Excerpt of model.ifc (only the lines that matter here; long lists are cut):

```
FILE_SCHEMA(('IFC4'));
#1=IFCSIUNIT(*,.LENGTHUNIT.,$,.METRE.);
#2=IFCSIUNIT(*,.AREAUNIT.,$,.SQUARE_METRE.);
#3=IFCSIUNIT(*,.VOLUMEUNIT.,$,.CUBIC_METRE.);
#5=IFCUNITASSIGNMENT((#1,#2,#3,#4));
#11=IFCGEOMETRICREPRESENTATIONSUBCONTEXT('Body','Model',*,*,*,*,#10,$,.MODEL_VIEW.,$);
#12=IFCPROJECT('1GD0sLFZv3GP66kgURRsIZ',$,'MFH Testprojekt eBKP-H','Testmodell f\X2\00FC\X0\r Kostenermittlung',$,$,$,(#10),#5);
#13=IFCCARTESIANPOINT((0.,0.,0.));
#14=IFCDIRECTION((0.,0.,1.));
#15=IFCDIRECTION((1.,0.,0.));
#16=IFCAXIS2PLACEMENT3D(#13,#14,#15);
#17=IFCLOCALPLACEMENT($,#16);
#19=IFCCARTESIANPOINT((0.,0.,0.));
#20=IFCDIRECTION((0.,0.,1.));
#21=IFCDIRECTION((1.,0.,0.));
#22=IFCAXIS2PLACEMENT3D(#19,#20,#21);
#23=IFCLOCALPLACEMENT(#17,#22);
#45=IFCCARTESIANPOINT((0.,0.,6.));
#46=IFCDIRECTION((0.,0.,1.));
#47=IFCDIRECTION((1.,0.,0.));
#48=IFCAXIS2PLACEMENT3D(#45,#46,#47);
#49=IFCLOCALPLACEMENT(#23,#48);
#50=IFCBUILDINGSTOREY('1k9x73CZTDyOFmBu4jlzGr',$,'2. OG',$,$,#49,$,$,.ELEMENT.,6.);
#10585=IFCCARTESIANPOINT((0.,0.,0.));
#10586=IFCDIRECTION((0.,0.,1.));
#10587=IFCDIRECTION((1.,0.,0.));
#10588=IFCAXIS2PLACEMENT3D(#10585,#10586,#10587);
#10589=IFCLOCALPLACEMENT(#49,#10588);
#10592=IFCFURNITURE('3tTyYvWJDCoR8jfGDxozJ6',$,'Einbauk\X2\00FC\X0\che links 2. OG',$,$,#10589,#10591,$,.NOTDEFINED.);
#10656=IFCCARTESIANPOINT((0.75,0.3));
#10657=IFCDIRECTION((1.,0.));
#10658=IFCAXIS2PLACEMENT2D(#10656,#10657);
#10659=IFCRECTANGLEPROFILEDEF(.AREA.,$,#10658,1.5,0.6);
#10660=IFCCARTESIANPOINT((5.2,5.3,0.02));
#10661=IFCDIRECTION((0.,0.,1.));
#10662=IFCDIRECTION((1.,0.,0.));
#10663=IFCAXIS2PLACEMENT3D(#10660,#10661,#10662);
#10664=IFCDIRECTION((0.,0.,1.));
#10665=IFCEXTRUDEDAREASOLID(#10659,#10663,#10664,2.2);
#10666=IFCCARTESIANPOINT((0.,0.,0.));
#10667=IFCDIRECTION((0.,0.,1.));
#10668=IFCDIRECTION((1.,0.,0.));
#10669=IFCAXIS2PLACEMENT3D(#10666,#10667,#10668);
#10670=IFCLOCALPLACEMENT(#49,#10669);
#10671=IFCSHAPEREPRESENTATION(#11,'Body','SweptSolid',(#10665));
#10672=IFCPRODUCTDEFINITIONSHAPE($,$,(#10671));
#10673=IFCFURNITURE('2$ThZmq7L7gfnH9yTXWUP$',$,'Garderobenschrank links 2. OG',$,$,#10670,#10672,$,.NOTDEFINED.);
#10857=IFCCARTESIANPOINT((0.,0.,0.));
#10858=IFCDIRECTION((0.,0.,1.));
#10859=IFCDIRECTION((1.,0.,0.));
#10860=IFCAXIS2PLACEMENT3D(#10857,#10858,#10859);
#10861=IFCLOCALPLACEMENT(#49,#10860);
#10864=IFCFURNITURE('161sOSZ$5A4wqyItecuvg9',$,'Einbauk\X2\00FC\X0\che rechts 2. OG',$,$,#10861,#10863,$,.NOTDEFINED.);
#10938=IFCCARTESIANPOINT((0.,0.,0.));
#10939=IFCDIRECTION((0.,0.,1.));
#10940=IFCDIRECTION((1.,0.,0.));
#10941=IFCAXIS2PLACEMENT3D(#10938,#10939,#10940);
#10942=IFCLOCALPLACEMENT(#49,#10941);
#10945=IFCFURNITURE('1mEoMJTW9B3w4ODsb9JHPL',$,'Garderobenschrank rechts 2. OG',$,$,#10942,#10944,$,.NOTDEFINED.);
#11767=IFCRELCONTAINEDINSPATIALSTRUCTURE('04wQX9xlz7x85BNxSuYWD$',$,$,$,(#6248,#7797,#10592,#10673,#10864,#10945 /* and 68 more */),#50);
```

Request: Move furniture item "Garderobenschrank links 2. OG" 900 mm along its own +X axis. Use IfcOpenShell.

```python
import ifcopenshell
import ifcopenshell.api.geometry
import ifcopenshell.util.placement

model = ifcopenshell.open("model.ifc")

item = model.by_id(10673)
matrix = ifcopenshell.util.placement.get_local_placement(item.ObjectPlacement)
matrix[:3, 3] += matrix[:3, 0] * 0.9
ifcopenshell.api.geometry.edit_object_placement(model, product=item, matrix=matrix, is_si=False)

print(ifcopenshell.util.placement.get_local_placement(item.ObjectPlacement).round(3) + 0.0)

model.write("model_rev.ifc")
```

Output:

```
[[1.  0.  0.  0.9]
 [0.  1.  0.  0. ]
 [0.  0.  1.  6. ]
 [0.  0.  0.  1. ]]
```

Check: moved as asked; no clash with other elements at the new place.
